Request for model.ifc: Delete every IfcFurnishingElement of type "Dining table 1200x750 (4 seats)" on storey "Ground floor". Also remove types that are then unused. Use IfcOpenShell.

First a look at what the model holds.

```python
import ifcopenshell
import ifcopenshell.util.element

model = ifcopenshell.open("model.ifc")
print(model.schema)
storey = next(s for s in model.by_type("IfcBuildingStorey") if s.Name == "Ground floor")
furniture = [e for e in ifcopenshell.util.element.get_decomposition(storey) if e.is_a("IfcFurnishingElement")]
seen = {}
for e in furniture:
    element_type = ifcopenshell.util.element.get_type(e)
    name = element_type.Name if element_type not in (None, e) else None
    seen[name] = seen.get(name, 0) + 1
for name, count in sorted(seen.items(), key=str):
    print(count, "x", name)
```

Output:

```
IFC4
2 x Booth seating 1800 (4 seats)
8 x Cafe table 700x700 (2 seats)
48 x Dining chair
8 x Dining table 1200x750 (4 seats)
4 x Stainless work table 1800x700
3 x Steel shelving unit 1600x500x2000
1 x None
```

```python
import ifcopenshell
import ifcopenshell.api.root
import ifcopenshell.util.element

model = ifcopenshell.open("model.ifc")

storey = next(s for s in model.by_type("IfcBuildingStorey") if s.Name == "Ground floor")
furniture = [e for e in ifcopenshell.util.element.get_decomposition(storey) if e.is_a("IfcFurnishingElement")]
targets = [e for e in furniture if (t := ifcopenshell.util.element.get_type(e)) not in (None, e) and t.Name == "Dining table 1200x750 (4 seats)"]
types = {ifcopenshell.util.element.get_type(e) for e in targets} - {None, *targets}

for e in targets:
    ifcopenshell.api.root.remove_product(model, product=e)
print(len(targets), "removed")

unused = [t for t in types if not ifcopenshell.util.element.get_types(t)]
for t in unused:
    ifcopenshell.api.root.remove_product(model, product=t)
print(len(unused), "unused types removed")

model.write("model-out.ifc")
```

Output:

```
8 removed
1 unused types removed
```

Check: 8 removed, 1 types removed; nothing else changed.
